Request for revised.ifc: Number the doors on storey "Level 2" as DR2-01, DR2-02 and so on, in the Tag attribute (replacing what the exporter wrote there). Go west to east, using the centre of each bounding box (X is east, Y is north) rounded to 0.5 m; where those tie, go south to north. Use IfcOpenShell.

First a look at what the model holds.

```python
import ifcopenshell
import ifcopenshell.util.element
import ifcopenshell.util.placement

model = ifcopenshell.open("revised.ifc")
print(model.schema)
storey = next(s for s in model.by_type("IfcBuildingStorey") if s.Name == "Level 2")
doors = [e for e in ifcopenshell.util.element.get_decomposition(storey) if e.is_a("IfcDoor")]
for e in sorted(doors, key=lambda e: e.id()):
    origin = ifcopenshell.util.placement.get_local_placement(e.ObjectPlacement)[:3, 3]
    print(e.id(), e.Tag, e.Name, origin.round(2) + 0.0, sep=" | ")
```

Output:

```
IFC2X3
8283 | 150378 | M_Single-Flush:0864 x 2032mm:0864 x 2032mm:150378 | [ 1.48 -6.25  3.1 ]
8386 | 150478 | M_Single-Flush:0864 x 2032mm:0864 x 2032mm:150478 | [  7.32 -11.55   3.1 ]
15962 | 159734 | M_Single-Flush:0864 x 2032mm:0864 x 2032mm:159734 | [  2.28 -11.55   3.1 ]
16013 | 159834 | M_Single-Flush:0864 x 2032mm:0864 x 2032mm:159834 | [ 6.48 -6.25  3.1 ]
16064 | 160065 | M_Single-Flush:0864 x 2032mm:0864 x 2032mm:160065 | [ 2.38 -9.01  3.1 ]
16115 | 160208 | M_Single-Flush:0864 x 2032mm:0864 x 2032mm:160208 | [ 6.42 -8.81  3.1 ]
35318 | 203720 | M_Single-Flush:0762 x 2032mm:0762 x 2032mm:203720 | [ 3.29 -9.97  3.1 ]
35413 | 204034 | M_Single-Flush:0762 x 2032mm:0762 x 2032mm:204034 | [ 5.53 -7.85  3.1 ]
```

```python
import ifcopenshell
import ifcopenshell.geom
import ifcopenshell.util.element
import ifcopenshell.util.shape

model = ifcopenshell.open("revised.ifc")
settings = ifcopenshell.geom.settings()
settings.set("use-world-coords", True)


def centre(element):
    shape = ifcopenshell.geom.create_shape(settings, element)
    return ifcopenshell.util.shape.get_bbox_centroid(shape.geometry)


storey = next(s for s in model.by_type("IfcBuildingStorey") if s.Name == "Level 2")
doors = [e for e in ifcopenshell.util.element.get_decomposition(storey) if e.is_a("IfcDoor")]

# Insertion points can sit at a corner or the storey origin, so sort by the geometry (in metres).
centres = {e: centre(e) for e in doors}
doors.sort(key=lambda e: (round(centres[e][0] / 0.5), centres[e][1]))

for i, e in enumerate(doors, start=1):
    number = f"DR2-{i:02d}"
    e.Tag = number
    print(e.id(), number)

model.write("revised_v2.ifc")
```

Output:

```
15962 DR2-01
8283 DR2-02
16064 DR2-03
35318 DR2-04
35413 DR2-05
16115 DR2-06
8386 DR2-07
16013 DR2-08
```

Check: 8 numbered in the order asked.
